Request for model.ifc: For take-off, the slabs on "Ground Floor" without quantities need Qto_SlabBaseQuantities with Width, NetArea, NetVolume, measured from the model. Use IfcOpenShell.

First a look at what the model holds.

```python
import ifcopenshell
import ifcopenshell.util.element
import ifcopenshell.util.unit

model = ifcopenshell.open("model.ifc")
print(model.schema)
for unit_type in ("LENGTHUNIT", "AREAUNIT", "VOLUMEUNIT"):
    print(unit_type, ifcopenshell.util.unit.calculate_unit_scale(model, unit_type))
storey = next(s for s in model.by_type("IfcBuildingStorey") if s.Name == "Ground Floor")
slabs = [e for e in ifcopenshell.util.element.get_decomposition(storey) if e.is_a("IfcSlab")]
for e in sorted(slabs, key=lambda e: e.id()):
    print(e.id(), e.is_a(), e.Name, list(ifcopenshell.util.element.get_psets(e, qtos_only=True)), sep=" | ")
```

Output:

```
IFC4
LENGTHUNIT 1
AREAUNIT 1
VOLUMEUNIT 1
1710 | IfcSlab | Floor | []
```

```python
import ifcopenshell
import ifcopenshell.api.pset
import ifcopenshell.geom
import ifcopenshell.util.element
import ifcopenshell.util.shape
import ifcopenshell.util.unit

model = ifcopenshell.open("model.ifc")
unit_scale = ifcopenshell.util.unit.calculate_unit_scale(model)
area_scale = ifcopenshell.util.unit.calculate_unit_scale(model, "AREAUNIT")
volume_scale = ifcopenshell.util.unit.calculate_unit_scale(model, "VOLUMEUNIT")
settings = ifcopenshell.geom.settings()

storey = next(s for s in model.by_type("IfcBuildingStorey") if s.Name == "Ground Floor")
slabs = [e for e in ifcopenshell.util.element.get_decomposition(storey) if e.is_a("IfcSlab")]

for e in sorted(slabs, key=lambda e: e.id()):
    if ifcopenshell.util.element.get_psets(e, qtos_only=True, should_inherit=False):
        continue
    # Geometry comes back in metres, in the element's own axes.
    shape = ifcopenshell.geom.create_shape(settings, e)
    values = {
        "Width": ifcopenshell.util.shape.get_z(shape.geometry) / unit_scale,
        "NetArea": ifcopenshell.util.shape.get_footprint_area(shape.geometry) / area_scale,
        "NetVolume": ifcopenshell.util.shape.get_volume(shape.geometry) / volume_scale,
    }
    qto = ifcopenshell.api.pset.add_qto(model, product=e, name="Qto_SlabBaseQuantities")
    ifcopenshell.api.pset.edit_qto(model, qto=qto, properties=values)
    print(e.id(), {k: round(v, 3) for k, v in values.items()})

model.write("model_rev.ifc")
```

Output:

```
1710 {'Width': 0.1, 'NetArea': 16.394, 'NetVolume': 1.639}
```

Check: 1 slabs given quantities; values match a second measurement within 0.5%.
